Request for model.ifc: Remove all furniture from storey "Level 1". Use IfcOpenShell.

First a look at what the model holds.

```python
import ifcopenshell
import ifcopenshell.util.element

model = ifcopenshell.open("model.ifc")
print(model.schema)
storey = next(s for s in model.by_type("IfcBuildingStorey") if s.Name == "Level 1")
furniture = [e for e in ifcopenshell.util.element.get_decomposition(storey) if e.is_a("IfcFurnishingElement")]
seen = {}
for e in furniture:
    element_type = ifcopenshell.util.element.get_type(e)
    name = element_type.Name if element_type not in (None, e) else None
    seen[name] = seen.get(name, 0) + 1
for name, count in sorted(seen.items(), key=str):
    print(count, "x", name)
```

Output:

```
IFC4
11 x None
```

```python
import ifcopenshell
import ifcopenshell.api.root
import ifcopenshell.util.element

model = ifcopenshell.open("model.ifc")

storey = next(s for s in model.by_type("IfcBuildingStorey") if s.Name == "Level 1")
furniture = [e for e in ifcopenshell.util.element.get_decomposition(storey) if e.is_a("IfcFurnishingElement")]

for e in furniture:
    ifcopenshell.api.root.remove_product(model, product=e)
print(len(furniture), "removed")

model.write("model_updated.ifc")
```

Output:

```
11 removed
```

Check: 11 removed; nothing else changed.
